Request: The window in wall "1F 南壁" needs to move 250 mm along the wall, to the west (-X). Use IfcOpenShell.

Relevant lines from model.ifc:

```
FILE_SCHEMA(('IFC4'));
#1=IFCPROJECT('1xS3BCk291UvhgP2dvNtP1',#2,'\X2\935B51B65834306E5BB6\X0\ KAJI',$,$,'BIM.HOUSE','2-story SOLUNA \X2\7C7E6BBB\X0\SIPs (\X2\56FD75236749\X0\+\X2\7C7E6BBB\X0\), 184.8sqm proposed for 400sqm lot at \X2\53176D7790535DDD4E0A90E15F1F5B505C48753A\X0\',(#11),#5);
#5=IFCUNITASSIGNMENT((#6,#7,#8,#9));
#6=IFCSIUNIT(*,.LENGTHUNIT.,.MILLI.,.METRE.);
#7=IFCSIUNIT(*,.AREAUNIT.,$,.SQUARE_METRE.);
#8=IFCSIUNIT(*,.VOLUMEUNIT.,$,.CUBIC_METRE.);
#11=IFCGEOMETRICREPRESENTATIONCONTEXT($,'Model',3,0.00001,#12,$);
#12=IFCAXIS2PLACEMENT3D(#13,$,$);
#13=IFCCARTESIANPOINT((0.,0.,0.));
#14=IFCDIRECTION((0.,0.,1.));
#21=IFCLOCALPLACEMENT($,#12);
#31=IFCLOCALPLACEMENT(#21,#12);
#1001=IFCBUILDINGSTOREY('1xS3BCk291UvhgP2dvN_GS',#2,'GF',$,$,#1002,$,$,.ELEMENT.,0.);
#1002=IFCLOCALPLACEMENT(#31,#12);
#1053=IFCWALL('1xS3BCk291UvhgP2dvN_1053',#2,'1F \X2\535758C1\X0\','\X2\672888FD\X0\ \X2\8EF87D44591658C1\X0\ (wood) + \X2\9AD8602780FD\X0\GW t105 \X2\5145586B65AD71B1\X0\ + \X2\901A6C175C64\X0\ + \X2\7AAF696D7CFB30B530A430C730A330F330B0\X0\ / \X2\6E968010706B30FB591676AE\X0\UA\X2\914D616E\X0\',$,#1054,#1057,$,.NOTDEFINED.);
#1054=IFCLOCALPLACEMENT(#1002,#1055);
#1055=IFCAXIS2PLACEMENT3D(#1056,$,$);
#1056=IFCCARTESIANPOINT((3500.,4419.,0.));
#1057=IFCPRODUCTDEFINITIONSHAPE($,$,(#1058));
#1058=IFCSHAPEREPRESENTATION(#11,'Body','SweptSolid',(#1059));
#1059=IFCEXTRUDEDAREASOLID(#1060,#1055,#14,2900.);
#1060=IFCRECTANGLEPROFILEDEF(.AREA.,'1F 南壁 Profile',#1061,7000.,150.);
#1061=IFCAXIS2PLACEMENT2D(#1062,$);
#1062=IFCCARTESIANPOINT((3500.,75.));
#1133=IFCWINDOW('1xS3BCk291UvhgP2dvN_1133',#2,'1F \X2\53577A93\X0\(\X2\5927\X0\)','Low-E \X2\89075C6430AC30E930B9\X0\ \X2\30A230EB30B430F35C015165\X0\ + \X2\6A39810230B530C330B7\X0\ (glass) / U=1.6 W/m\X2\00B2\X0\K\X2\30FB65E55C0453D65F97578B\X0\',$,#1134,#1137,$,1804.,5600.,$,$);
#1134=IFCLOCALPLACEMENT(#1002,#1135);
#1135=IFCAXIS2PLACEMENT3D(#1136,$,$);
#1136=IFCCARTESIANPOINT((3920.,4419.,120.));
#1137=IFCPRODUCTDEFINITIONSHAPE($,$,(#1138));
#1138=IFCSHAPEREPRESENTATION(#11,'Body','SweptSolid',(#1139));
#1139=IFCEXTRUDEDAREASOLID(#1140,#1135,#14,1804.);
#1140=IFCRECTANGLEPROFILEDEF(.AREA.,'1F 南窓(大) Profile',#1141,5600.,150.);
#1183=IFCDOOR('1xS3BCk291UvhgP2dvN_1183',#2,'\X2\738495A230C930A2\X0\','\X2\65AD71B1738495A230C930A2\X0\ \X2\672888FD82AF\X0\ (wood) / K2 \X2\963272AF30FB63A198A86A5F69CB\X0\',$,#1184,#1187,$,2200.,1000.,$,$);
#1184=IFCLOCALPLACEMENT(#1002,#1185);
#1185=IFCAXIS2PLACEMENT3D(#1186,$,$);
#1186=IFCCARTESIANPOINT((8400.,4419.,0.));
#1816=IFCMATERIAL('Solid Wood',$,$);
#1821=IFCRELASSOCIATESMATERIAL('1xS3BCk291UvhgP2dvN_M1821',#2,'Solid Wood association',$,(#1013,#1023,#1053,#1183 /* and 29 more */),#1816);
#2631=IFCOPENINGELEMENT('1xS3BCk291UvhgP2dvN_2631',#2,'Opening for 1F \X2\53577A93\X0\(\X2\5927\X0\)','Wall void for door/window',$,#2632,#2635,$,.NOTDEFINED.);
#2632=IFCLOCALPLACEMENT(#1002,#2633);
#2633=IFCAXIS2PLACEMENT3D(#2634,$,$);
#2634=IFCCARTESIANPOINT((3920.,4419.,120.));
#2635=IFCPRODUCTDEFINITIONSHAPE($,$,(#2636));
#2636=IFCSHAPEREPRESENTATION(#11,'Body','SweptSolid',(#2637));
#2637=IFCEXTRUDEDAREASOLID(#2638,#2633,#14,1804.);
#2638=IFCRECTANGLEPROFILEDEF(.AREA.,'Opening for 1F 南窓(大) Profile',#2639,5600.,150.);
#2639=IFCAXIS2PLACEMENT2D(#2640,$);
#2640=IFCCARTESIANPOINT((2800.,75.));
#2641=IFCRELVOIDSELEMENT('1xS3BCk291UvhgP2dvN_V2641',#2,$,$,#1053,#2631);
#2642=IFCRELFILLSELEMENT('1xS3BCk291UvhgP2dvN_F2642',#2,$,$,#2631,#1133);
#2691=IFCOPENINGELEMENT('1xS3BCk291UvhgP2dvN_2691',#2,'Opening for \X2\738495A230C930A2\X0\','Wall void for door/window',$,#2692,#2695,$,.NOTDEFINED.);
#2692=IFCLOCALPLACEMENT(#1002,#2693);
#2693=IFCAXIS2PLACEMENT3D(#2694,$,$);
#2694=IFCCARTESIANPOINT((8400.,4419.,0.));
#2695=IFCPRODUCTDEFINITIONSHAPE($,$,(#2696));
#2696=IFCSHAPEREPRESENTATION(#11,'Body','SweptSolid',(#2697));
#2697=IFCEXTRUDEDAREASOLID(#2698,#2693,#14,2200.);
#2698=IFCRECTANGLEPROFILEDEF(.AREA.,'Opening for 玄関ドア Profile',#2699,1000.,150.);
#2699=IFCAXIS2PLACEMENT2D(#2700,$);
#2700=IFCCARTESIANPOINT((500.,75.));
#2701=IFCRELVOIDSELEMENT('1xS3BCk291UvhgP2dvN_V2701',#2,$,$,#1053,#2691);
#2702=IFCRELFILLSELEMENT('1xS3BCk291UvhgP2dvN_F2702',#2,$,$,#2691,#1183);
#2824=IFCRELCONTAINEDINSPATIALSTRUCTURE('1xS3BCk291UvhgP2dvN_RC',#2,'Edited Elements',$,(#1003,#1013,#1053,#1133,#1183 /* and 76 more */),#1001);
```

```python
import ifcopenshell
import ifcopenshell.api.geometry
import ifcopenshell.util.placement
import ifcopenshell.util.unit

model = ifcopenshell.open("model.ifc")
unit_scale = ifcopenshell.util.unit.calculate_unit_scale(model)

window = model.by_guid("1xS3BCk291UvhgP2dvN_1133")
opening = window.FillsVoids[0].RelatingOpeningElement
wall = opening.VoidsElements[0].RelatingBuildingElement

wall_matrix = ifcopenshell.util.placement.get_local_placement(wall.ObjectPlacement)
shift = wall_matrix[:3, 0] * -0.25 / unit_scale
before = ifcopenshell.util.placement.get_local_placement(window.ObjectPlacement)[:3, 3].copy()

# The window is not placed relative to its opening, so move both.
for product in (opening, window):
    matrix = ifcopenshell.util.placement.get_local_placement(product.ObjectPlacement)
    matrix[:3, 3] += shift
    ifcopenshell.api.geometry.edit_object_placement(model, product=product, matrix=matrix, is_si=False)

after = ifcopenshell.util.placement.get_local_placement(window.ObjectPlacement)[:3, 3]
print("window moved by", (after - before).round(3) + 0.0)

model.write("model_updated.ifc")
```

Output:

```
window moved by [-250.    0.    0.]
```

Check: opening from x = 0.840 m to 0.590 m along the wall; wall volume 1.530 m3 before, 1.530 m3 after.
